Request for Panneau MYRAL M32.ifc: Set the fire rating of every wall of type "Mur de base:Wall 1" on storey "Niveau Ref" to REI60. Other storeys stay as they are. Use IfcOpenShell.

First a look at what the model holds.

```python
import ifcopenshell
import ifcopenshell.util.element

model = ifcopenshell.open("Panneau MYRAL M32.ifc")
print(model.schema)
storey = next(s for s in model.by_type("IfcBuildingStorey") if s.Name == "Niveau Ref")
walls = [e for e in ifcopenshell.util.element.get_decomposition(storey) if e.is_a("IfcWall")]
seen = {}
for e in walls:
    element_type = ifcopenshell.util.element.get_type(e)
    key = (element_type.Name if element_type != e and element_type else None, ifcopenshell.util.element.get_pset(e, "Pset_WallCommon", "FireRating"))
    seen[key] = seen.get(key, 0) + 1
for (name, value), count in sorted(seen.items(), key=str):
    print(count, "x", name, "|", value)
```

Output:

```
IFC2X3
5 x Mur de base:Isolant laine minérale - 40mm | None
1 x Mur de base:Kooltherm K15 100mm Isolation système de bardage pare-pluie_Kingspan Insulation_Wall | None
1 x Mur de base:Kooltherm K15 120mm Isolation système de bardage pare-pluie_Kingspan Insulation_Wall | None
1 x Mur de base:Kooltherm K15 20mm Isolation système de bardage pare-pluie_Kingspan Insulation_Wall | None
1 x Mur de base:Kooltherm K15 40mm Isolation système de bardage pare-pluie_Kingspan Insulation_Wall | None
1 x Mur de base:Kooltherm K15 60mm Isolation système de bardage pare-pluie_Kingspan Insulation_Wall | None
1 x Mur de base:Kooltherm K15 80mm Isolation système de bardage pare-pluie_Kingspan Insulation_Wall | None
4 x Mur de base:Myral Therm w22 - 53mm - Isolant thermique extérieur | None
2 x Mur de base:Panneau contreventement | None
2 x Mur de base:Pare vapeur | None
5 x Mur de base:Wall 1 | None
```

```python
import ifcopenshell
import ifcopenshell.api.pset
import ifcopenshell.util.element

model = ifcopenshell.open("Panneau MYRAL M32.ifc")

storey = next(s for s in model.by_type("IfcBuildingStorey") if s.Name == "Niveau Ref")
walls = [e for e in ifcopenshell.util.element.get_decomposition(storey) if e.is_a("IfcWall")]

count = 0
for e in walls:
    element_type = ifcopenshell.util.element.get_type(e)
    if element_type in (None, e) or element_type.Name != "Mur de base:Wall 1":
        continue
    # add_pset returns the element's existing set when there is one.
    pset = ifcopenshell.api.pset.add_pset(model, product=e, name="Pset_WallCommon")
    ifcopenshell.api.pset.edit_pset(model, pset=pset, properties={"FireRating": "REI60"})
    count += 1

print(count, "walls updated")

model.write("Panneau MYRAL M32_rev.ifc")
```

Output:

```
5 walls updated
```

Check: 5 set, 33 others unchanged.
